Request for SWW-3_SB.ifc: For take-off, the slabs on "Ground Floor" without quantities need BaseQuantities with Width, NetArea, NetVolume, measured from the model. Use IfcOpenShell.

First a look at what the model holds.

```python
import ifcopenshell
import ifcopenshell.util.element
import ifcopenshell.util.unit

model = ifcopenshell.open("SWW-3_SB.ifc")
print(model.schema)
for unit_type in ("LENGTHUNIT", "AREAUNIT", "VOLUMEUNIT"):
    print(unit_type, ifcopenshell.util.unit.calculate_unit_scale(model, unit_type))
storey = next(s for s in model.by_type("IfcBuildingStorey") if s.Name == "Ground Floor")
slabs = [e for e in ifcopenshell.util.element.get_decomposition(storey) if e.is_a("IfcSlab")]
for e in sorted(slabs, key=lambda e: e.id()):
    print(e.id(), e.is_a(), e.Name, list(ifcopenshell.util.element.get_psets(e, qtos_only=True)), sep=" | ")
```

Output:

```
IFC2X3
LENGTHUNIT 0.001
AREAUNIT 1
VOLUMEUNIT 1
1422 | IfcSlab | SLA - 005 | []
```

```python
import ifcopenshell
import ifcopenshell.api.pset
import ifcopenshell.geom
import ifcopenshell.util.element
import ifcopenshell.util.shape
import ifcopenshell.util.unit

model = ifcopenshell.open("SWW-3_SB.ifc")
unit_scale = ifcopenshell.util.unit.calculate_unit_scale(model)
area_scale = ifcopenshell.util.unit.calculate_unit_scale(model, "AREAUNIT")
volume_scale = ifcopenshell.util.unit.calculate_unit_scale(model, "VOLUMEUNIT")
settings = ifcopenshell.geom.settings()

storey = next(s for s in model.by_type("IfcBuildingStorey") if s.Name == "Ground Floor")
slabs = [e for e in ifcopenshell.util.element.get_decomposition(storey) if e.is_a("IfcSlab")]

for e in sorted(slabs, key=lambda e: e.id()):
    if ifcopenshell.util.element.get_psets(e, qtos_only=True, should_inherit=False):
        continue
    # Geometry comes back in metres, in the element's own axes.
    shape = ifcopenshell.geom.create_shape(settings, e)
    values = {
        "Width": ifcopenshell.util.shape.get_z(shape.geometry) / unit_scale,
        "NetArea": ifcopenshell.util.shape.get_footprint_area(shape.geometry) / area_scale,
        "NetVolume": ifcopenshell.util.shape.get_volume(shape.geometry) / volume_scale,
    }
    qto = ifcopenshell.api.pset.add_qto(model, product=e, name="BaseQuantities")
    ifcopenshell.api.pset.edit_qto(model, qto=qto, properties=values)
    print(e.id(), {k: round(v, 3) for k, v in values.items()})

model.write("SWW-3_SB_rev.ifc")
```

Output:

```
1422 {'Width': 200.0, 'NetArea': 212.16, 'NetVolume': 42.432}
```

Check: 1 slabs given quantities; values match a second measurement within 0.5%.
